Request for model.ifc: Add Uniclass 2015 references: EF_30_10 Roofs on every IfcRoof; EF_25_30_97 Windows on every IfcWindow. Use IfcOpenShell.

First a look at what the model holds.

```python
import ifcopenshell

model = ifcopenshell.open("model.ifc")
print(model.schema)
print("classifications:", [c.Name for c in model.by_type("IfcClassification")])
for ifc_class in ("IfcDoor", "IfcRoof", "IfcStair", "IfcWall", "IfcWindow"):
    print(ifc_class, len(model.by_type(ifc_class)))
```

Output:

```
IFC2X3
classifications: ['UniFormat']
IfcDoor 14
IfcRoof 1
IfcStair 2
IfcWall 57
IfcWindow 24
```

```python
import ifcopenshell
import ifcopenshell.api.classification

model = ifcopenshell.open("model.ifc")

# IFC2X3 requires Source and Edition and has no link from the project to the system.
system = model.create_entity("IfcClassification", Source="NBS", Edition="2015", Name="Uniclass 2015")

codes = {
    "IfcRoof": ("EF_30_10", "Roofs"),
    "IfcWindow": ("EF_25_30_97", "Windows"),
}
for ifc_class, (code, name) in codes.items():
    products = model.by_type(ifc_class)
    ifcopenshell.api.classification.add_reference(
        model, products=products, classification=system, identification=code, name=name
    )
    print(code, len(products))

model.write("model_v2.ifc")
```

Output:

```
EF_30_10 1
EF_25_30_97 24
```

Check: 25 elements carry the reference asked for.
